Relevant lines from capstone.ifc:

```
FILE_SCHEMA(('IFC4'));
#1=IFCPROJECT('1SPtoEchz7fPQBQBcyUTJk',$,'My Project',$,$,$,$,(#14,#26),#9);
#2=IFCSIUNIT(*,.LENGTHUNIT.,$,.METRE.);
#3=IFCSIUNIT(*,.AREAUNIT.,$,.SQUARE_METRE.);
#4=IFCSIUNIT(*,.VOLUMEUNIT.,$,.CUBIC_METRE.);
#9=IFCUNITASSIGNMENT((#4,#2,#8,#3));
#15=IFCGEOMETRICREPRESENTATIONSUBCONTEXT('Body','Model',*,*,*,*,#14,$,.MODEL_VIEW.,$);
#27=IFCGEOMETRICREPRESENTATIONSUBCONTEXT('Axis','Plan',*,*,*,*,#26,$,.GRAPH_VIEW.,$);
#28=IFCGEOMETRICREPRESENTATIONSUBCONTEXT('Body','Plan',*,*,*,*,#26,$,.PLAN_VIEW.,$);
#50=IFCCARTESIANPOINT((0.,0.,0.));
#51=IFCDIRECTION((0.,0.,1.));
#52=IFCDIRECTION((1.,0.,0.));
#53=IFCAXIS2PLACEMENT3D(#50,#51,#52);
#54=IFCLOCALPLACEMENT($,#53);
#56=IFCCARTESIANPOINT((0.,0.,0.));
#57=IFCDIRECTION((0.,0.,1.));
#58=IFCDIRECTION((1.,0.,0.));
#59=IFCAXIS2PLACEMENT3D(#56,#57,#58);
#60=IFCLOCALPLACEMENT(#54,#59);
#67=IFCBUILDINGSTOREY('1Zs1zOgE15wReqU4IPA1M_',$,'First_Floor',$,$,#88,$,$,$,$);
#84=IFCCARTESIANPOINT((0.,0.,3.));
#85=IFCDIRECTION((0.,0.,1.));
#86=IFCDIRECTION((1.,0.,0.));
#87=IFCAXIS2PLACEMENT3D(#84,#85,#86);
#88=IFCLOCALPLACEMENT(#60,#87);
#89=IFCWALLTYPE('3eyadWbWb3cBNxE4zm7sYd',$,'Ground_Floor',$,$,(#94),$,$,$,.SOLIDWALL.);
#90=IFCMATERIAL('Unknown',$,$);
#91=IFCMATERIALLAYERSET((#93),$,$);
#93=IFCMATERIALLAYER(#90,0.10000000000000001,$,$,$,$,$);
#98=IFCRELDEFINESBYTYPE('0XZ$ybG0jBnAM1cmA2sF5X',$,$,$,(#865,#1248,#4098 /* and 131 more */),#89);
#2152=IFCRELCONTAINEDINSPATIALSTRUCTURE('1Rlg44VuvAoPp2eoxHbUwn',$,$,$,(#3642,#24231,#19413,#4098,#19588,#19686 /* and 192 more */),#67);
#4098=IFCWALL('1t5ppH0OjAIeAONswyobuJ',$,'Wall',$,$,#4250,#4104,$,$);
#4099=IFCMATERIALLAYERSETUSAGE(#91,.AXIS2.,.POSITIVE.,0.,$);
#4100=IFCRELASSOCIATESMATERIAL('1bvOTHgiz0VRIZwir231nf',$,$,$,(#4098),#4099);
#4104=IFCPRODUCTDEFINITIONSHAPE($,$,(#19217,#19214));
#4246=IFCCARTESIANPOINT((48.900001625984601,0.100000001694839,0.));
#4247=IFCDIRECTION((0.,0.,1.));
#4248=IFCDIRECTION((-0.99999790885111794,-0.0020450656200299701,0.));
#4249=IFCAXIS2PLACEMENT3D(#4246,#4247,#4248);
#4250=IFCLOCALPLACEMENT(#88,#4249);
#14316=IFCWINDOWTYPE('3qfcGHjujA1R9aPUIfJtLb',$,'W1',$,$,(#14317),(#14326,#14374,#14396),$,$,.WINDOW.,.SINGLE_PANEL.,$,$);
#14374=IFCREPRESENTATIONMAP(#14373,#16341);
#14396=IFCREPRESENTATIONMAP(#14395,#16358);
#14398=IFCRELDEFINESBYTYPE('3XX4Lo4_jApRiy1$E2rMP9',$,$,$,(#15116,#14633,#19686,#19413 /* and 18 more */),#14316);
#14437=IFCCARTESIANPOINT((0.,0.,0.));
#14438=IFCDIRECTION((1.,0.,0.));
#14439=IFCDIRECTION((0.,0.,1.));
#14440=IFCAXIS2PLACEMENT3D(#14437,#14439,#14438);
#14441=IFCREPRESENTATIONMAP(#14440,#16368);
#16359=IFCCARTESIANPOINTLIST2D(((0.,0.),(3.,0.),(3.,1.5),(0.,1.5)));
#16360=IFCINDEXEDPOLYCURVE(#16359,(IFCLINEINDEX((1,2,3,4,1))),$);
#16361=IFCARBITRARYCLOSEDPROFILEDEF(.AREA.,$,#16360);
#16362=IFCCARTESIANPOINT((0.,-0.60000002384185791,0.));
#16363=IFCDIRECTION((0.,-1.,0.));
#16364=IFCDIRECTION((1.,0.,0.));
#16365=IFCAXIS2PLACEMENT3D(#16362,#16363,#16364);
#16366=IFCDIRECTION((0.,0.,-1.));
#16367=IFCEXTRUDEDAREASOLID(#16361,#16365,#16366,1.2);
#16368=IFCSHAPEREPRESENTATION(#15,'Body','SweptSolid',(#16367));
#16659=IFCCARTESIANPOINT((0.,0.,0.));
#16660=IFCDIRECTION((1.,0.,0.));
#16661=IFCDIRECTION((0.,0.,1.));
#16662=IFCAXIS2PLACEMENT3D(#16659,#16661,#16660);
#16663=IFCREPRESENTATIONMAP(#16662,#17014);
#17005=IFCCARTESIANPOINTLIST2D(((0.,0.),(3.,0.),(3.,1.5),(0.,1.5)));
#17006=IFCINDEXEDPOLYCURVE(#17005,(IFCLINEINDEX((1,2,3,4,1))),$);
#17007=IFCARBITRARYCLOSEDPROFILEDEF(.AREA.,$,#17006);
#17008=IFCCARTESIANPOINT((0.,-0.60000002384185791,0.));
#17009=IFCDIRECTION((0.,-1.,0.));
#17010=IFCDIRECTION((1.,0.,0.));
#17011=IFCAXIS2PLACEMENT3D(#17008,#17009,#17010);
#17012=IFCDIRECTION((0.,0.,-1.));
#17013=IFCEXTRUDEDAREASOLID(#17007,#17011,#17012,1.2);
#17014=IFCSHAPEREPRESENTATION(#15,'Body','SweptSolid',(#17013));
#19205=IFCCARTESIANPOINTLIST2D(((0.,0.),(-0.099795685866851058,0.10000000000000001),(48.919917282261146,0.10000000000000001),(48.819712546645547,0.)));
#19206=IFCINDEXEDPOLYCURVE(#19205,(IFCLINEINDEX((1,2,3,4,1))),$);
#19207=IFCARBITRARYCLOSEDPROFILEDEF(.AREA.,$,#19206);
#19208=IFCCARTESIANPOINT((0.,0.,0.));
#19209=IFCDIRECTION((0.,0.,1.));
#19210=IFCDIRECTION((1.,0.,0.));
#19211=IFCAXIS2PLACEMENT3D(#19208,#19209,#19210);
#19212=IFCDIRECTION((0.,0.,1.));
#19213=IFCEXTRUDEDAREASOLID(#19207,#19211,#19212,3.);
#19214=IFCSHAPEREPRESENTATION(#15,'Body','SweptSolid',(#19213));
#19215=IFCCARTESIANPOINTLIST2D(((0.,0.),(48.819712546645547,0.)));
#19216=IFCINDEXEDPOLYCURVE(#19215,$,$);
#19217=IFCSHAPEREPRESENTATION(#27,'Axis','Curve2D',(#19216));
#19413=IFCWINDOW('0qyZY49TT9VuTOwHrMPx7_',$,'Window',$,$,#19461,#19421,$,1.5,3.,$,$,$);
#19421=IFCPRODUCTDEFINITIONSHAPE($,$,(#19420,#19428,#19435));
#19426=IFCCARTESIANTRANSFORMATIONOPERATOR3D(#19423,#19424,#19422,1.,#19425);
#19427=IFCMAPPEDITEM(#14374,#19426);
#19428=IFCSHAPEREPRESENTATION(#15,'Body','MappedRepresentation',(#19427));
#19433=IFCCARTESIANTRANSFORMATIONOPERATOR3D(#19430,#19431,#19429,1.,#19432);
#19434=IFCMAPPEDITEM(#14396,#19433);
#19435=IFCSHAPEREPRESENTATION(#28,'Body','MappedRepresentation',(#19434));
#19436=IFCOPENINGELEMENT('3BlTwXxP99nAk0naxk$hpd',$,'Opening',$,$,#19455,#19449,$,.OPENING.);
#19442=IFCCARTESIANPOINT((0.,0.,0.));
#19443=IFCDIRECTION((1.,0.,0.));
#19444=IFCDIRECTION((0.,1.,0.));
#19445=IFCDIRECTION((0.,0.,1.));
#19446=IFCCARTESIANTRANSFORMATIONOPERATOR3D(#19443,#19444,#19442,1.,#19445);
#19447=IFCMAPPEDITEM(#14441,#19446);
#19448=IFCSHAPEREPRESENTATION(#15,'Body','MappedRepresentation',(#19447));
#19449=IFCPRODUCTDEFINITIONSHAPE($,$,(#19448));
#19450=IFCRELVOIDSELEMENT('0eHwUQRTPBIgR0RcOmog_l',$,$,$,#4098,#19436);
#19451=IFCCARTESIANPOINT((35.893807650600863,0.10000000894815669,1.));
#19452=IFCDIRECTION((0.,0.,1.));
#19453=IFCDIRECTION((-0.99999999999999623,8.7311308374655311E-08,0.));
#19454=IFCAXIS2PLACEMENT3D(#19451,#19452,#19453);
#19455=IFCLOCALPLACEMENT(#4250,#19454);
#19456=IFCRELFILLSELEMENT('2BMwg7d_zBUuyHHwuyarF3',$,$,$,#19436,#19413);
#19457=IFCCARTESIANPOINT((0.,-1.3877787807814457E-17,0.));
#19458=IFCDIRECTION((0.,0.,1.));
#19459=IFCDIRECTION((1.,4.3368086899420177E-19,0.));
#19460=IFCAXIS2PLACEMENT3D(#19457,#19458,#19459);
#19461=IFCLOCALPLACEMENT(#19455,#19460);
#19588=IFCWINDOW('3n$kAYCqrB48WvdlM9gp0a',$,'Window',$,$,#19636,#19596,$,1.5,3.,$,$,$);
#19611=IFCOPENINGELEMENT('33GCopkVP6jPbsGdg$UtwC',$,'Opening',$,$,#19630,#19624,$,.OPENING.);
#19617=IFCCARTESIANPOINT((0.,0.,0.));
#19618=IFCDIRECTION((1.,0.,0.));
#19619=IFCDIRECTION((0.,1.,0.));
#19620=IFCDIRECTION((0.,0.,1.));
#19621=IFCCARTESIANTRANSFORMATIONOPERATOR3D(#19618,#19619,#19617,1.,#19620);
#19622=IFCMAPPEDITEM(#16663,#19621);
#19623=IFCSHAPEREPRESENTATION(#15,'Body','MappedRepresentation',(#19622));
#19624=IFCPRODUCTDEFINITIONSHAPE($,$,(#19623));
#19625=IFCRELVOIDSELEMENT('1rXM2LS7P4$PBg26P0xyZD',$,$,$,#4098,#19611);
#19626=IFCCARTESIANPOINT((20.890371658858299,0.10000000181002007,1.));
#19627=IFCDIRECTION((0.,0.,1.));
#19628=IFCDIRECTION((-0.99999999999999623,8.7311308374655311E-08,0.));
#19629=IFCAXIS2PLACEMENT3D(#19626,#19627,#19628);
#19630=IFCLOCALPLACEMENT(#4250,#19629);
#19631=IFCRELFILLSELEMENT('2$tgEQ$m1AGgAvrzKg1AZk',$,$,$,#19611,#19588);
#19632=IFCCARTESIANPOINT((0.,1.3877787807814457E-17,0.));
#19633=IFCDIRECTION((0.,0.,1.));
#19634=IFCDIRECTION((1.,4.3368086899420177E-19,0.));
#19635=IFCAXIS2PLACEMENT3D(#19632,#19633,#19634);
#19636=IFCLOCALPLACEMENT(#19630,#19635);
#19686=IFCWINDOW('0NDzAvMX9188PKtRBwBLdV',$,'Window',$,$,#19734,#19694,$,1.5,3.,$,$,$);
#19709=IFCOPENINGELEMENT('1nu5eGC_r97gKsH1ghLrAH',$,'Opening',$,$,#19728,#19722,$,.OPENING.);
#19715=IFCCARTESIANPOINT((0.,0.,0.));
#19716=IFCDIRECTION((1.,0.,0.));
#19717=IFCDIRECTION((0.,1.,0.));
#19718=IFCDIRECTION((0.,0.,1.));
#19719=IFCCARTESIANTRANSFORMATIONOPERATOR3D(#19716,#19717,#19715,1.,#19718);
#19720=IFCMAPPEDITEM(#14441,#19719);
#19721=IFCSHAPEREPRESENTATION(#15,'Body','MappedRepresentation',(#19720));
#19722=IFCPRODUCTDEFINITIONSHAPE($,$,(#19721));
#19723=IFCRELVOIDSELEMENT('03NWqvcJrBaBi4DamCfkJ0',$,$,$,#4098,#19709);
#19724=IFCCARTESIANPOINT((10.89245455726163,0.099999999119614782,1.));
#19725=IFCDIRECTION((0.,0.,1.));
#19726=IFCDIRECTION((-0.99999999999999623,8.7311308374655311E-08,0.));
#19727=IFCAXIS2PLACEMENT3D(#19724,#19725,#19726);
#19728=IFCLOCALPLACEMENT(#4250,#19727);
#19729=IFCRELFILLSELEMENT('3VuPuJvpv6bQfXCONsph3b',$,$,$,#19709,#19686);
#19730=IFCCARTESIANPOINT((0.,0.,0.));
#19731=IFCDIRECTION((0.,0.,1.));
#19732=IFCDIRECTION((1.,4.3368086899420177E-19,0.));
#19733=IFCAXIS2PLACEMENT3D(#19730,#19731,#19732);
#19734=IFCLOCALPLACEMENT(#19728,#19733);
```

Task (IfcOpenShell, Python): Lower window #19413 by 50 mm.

```python
import numpy as np
import ifcopenshell
import ifcopenshell.api.geometry
import ifcopenshell.util.placement
import ifcopenshell.util.unit

model = ifcopenshell.open("capstone.ifc")
unit_scale = ifcopenshell.util.unit.calculate_unit_scale(model)

window = model.by_id(19413)
opening = window.FillsVoids[0].RelatingOpeningElement
dz = -0.05

shift = np.array([0.0, 0.0, dz])
# The window is placed relative to its opening, so it follows when the opening moves.
matrix = ifcopenshell.util.placement.get_local_placement(opening.ObjectPlacement)
matrix[:3, 3] += shift
ifcopenshell.api.geometry.edit_object_placement(
    model, product=opening, matrix=matrix, is_si=False, should_transform_children=True
)

print(f"moved by {dz * unit_scale:+.3f} m")

model.write("capstone_edited.ifc")
```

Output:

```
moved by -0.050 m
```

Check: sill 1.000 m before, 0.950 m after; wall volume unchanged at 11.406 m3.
